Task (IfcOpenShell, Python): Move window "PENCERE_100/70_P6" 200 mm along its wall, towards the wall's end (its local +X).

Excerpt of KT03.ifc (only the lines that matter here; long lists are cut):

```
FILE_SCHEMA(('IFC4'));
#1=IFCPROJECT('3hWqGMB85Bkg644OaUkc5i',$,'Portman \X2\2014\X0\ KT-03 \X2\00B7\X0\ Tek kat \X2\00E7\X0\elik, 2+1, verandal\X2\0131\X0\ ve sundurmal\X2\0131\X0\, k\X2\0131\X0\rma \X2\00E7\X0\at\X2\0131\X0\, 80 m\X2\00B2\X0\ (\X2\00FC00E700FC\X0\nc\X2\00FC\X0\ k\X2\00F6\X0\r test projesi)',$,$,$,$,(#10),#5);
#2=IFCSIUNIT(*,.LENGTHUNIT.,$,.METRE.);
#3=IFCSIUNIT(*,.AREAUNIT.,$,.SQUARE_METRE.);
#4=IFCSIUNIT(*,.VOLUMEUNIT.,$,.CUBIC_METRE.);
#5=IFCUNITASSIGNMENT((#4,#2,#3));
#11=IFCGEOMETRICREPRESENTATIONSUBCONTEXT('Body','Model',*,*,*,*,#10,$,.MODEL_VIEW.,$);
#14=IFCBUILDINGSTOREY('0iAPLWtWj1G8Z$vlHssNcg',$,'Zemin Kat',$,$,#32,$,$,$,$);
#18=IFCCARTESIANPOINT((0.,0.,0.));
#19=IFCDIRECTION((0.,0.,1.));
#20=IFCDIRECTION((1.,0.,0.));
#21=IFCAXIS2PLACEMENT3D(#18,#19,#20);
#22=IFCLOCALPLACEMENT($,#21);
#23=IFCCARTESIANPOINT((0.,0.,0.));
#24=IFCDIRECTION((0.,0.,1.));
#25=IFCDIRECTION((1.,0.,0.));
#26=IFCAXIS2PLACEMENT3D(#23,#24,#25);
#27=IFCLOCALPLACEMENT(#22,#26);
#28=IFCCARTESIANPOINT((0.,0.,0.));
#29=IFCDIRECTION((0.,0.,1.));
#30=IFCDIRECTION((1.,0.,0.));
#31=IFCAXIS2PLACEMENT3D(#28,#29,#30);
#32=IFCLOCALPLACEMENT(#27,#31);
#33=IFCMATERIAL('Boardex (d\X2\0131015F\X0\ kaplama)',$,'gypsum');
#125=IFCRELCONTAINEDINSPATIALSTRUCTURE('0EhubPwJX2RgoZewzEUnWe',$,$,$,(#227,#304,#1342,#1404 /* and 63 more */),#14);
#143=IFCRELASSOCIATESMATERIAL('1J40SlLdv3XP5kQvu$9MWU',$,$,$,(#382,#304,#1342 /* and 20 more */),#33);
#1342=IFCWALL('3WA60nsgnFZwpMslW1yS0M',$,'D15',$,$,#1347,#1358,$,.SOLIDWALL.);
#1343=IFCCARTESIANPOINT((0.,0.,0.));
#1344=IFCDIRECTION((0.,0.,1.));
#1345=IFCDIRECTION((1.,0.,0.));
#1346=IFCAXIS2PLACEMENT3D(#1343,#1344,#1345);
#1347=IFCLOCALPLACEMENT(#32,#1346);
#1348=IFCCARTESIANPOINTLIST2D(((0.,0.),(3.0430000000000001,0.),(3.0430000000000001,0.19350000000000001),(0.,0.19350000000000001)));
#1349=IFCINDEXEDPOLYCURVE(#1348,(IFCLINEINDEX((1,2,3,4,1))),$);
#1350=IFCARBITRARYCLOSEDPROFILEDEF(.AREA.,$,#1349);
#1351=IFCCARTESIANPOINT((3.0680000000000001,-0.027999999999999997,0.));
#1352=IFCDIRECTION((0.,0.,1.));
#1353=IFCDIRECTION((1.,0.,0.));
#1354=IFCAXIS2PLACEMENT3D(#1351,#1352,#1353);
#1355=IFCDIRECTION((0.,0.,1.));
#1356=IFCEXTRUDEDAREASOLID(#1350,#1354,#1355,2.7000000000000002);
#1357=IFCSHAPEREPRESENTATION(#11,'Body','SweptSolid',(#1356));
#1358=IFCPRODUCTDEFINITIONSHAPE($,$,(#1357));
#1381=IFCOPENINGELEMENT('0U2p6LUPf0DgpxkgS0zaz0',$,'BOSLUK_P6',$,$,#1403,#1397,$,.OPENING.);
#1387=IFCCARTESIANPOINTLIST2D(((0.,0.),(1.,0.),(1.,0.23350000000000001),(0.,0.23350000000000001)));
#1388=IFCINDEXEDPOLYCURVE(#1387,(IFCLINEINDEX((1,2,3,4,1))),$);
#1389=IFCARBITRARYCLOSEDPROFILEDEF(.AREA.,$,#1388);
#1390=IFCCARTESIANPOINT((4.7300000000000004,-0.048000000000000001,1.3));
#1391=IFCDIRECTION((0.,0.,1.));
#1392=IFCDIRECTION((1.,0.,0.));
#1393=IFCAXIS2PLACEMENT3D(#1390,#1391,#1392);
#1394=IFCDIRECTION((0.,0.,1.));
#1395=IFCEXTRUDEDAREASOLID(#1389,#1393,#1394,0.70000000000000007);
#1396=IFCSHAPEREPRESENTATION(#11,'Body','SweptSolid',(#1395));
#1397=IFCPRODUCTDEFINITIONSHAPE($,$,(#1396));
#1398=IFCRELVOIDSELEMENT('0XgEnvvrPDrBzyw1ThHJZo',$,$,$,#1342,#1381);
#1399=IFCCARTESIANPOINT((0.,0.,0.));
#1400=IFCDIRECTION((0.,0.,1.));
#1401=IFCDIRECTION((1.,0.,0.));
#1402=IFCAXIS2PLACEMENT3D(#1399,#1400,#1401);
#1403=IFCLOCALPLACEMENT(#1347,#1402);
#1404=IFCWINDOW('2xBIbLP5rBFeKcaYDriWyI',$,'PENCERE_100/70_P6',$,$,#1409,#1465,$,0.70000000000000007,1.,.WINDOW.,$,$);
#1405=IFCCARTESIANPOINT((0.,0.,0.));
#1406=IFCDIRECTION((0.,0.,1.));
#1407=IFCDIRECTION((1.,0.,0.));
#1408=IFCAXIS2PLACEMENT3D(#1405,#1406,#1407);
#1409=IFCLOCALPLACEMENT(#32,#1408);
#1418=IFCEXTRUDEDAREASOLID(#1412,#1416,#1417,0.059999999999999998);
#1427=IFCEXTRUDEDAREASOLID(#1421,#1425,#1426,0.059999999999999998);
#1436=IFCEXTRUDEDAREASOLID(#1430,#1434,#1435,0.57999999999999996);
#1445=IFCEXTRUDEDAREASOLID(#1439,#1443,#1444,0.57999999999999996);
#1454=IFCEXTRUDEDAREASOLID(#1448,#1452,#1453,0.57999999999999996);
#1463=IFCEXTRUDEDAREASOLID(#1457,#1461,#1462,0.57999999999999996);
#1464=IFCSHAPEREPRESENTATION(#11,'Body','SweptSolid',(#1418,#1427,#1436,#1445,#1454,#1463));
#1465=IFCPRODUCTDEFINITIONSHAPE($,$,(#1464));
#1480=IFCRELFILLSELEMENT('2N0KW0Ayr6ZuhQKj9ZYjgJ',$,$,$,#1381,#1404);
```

```python
import ifcopenshell
import ifcopenshell.api.geometry
import ifcopenshell.util.placement
import ifcopenshell.util.unit

model = ifcopenshell.open("KT03.ifc")
unit_scale = ifcopenshell.util.unit.calculate_unit_scale(model)

window = model.by_guid("2xBIbLP5rBFeKcaYDriWyI")
opening = window.FillsVoids[0].RelatingOpeningElement
wall = opening.VoidsElements[0].RelatingBuildingElement

wall_matrix = ifcopenshell.util.placement.get_local_placement(wall.ObjectPlacement)
shift = wall_matrix[:3, 0] * 0.2 / unit_scale
before = ifcopenshell.util.placement.get_local_placement(window.ObjectPlacement)[:3, 3].copy()

# The window is not placed relative to its opening, so move both.
for product in (opening, window):
    matrix = ifcopenshell.util.placement.get_local_placement(product.ObjectPlacement)
    matrix[:3, 3] += shift
    ifcopenshell.api.geometry.edit_object_placement(model, product=product, matrix=matrix, is_si=False)

after = ifcopenshell.util.placement.get_local_placement(window.ObjectPlacement)[:3, 3]
print("window moved by", (after - before).round(3) + 0.0)

model.write("KT03_updated.ifc")
```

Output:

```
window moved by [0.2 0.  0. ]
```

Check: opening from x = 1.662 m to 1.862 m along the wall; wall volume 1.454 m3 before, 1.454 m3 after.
